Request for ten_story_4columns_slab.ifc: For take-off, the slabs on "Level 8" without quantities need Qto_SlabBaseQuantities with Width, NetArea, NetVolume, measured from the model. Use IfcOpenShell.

First a look at what the model holds.

```python
import ifcopenshell
import ifcopenshell.util.element
import ifcopenshell.util.unit

model = ifcopenshell.open("ten_story_4columns_slab.ifc")
print(model.schema)
for unit_type in ("LENGTHUNIT", "AREAUNIT", "VOLUMEUNIT"):
    print(unit_type, ifcopenshell.util.unit.calculate_unit_scale(model, unit_type))
storey = next(s for s in model.by_type("IfcBuildingStorey") if s.Name == "Level 8")
slabs = [e for e in ifcopenshell.util.element.get_decomposition(storey) if e.is_a("IfcSlab")]
for e in sorted(slabs, key=lambda e: e.id()):
    print(e.id(), e.is_a(), e.Name, list(ifcopenshell.util.element.get_psets(e, qtos_only=True)), sep=" | ")
```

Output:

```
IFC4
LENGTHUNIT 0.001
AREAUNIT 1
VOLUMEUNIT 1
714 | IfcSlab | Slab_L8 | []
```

```python
import ifcopenshell
import ifcopenshell.api.pset
import ifcopenshell.geom
import ifcopenshell.util.element
import ifcopenshell.util.shape
import ifcopenshell.util.unit

model = ifcopenshell.open("ten_story_4columns_slab.ifc")
unit_scale = ifcopenshell.util.unit.calculate_unit_scale(model)
area_scale = ifcopenshell.util.unit.calculate_unit_scale(model, "AREAUNIT")
volume_scale = ifcopenshell.util.unit.calculate_unit_scale(model, "VOLUMEUNIT")
settings = ifcopenshell.geom.settings()

storey = next(s for s in model.by_type("IfcBuildingStorey") if s.Name == "Level 8")
slabs = [e for e in ifcopenshell.util.element.get_decomposition(storey) if e.is_a("IfcSlab")]

for e in sorted(slabs, key=lambda e: e.id()):
    if ifcopenshell.util.element.get_psets(e, qtos_only=True, should_inherit=False):
        continue
    # Geometry comes back in metres, in the element's own axes.
    shape = ifcopenshell.geom.create_shape(settings, e)
    values = {
        "Width": ifcopenshell.util.shape.get_z(shape.geometry) / unit_scale,
        "NetArea": ifcopenshell.util.shape.get_footprint_area(shape.geometry) / area_scale,
        "NetVolume": ifcopenshell.util.shape.get_volume(shape.geometry) / volume_scale,
    }
    qto = ifcopenshell.api.pset.add_qto(model, product=e, name="Qto_SlabBaseQuantities")
    ifcopenshell.api.pset.edit_qto(model, qto=qto, properties=values)
    print(e.id(), {k: round(v, 3) for k, v in values.items()})

model.write("ten_story_4columns_slab_v2.ifc")
```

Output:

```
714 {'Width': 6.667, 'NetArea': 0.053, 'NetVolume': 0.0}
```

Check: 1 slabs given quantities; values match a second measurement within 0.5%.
